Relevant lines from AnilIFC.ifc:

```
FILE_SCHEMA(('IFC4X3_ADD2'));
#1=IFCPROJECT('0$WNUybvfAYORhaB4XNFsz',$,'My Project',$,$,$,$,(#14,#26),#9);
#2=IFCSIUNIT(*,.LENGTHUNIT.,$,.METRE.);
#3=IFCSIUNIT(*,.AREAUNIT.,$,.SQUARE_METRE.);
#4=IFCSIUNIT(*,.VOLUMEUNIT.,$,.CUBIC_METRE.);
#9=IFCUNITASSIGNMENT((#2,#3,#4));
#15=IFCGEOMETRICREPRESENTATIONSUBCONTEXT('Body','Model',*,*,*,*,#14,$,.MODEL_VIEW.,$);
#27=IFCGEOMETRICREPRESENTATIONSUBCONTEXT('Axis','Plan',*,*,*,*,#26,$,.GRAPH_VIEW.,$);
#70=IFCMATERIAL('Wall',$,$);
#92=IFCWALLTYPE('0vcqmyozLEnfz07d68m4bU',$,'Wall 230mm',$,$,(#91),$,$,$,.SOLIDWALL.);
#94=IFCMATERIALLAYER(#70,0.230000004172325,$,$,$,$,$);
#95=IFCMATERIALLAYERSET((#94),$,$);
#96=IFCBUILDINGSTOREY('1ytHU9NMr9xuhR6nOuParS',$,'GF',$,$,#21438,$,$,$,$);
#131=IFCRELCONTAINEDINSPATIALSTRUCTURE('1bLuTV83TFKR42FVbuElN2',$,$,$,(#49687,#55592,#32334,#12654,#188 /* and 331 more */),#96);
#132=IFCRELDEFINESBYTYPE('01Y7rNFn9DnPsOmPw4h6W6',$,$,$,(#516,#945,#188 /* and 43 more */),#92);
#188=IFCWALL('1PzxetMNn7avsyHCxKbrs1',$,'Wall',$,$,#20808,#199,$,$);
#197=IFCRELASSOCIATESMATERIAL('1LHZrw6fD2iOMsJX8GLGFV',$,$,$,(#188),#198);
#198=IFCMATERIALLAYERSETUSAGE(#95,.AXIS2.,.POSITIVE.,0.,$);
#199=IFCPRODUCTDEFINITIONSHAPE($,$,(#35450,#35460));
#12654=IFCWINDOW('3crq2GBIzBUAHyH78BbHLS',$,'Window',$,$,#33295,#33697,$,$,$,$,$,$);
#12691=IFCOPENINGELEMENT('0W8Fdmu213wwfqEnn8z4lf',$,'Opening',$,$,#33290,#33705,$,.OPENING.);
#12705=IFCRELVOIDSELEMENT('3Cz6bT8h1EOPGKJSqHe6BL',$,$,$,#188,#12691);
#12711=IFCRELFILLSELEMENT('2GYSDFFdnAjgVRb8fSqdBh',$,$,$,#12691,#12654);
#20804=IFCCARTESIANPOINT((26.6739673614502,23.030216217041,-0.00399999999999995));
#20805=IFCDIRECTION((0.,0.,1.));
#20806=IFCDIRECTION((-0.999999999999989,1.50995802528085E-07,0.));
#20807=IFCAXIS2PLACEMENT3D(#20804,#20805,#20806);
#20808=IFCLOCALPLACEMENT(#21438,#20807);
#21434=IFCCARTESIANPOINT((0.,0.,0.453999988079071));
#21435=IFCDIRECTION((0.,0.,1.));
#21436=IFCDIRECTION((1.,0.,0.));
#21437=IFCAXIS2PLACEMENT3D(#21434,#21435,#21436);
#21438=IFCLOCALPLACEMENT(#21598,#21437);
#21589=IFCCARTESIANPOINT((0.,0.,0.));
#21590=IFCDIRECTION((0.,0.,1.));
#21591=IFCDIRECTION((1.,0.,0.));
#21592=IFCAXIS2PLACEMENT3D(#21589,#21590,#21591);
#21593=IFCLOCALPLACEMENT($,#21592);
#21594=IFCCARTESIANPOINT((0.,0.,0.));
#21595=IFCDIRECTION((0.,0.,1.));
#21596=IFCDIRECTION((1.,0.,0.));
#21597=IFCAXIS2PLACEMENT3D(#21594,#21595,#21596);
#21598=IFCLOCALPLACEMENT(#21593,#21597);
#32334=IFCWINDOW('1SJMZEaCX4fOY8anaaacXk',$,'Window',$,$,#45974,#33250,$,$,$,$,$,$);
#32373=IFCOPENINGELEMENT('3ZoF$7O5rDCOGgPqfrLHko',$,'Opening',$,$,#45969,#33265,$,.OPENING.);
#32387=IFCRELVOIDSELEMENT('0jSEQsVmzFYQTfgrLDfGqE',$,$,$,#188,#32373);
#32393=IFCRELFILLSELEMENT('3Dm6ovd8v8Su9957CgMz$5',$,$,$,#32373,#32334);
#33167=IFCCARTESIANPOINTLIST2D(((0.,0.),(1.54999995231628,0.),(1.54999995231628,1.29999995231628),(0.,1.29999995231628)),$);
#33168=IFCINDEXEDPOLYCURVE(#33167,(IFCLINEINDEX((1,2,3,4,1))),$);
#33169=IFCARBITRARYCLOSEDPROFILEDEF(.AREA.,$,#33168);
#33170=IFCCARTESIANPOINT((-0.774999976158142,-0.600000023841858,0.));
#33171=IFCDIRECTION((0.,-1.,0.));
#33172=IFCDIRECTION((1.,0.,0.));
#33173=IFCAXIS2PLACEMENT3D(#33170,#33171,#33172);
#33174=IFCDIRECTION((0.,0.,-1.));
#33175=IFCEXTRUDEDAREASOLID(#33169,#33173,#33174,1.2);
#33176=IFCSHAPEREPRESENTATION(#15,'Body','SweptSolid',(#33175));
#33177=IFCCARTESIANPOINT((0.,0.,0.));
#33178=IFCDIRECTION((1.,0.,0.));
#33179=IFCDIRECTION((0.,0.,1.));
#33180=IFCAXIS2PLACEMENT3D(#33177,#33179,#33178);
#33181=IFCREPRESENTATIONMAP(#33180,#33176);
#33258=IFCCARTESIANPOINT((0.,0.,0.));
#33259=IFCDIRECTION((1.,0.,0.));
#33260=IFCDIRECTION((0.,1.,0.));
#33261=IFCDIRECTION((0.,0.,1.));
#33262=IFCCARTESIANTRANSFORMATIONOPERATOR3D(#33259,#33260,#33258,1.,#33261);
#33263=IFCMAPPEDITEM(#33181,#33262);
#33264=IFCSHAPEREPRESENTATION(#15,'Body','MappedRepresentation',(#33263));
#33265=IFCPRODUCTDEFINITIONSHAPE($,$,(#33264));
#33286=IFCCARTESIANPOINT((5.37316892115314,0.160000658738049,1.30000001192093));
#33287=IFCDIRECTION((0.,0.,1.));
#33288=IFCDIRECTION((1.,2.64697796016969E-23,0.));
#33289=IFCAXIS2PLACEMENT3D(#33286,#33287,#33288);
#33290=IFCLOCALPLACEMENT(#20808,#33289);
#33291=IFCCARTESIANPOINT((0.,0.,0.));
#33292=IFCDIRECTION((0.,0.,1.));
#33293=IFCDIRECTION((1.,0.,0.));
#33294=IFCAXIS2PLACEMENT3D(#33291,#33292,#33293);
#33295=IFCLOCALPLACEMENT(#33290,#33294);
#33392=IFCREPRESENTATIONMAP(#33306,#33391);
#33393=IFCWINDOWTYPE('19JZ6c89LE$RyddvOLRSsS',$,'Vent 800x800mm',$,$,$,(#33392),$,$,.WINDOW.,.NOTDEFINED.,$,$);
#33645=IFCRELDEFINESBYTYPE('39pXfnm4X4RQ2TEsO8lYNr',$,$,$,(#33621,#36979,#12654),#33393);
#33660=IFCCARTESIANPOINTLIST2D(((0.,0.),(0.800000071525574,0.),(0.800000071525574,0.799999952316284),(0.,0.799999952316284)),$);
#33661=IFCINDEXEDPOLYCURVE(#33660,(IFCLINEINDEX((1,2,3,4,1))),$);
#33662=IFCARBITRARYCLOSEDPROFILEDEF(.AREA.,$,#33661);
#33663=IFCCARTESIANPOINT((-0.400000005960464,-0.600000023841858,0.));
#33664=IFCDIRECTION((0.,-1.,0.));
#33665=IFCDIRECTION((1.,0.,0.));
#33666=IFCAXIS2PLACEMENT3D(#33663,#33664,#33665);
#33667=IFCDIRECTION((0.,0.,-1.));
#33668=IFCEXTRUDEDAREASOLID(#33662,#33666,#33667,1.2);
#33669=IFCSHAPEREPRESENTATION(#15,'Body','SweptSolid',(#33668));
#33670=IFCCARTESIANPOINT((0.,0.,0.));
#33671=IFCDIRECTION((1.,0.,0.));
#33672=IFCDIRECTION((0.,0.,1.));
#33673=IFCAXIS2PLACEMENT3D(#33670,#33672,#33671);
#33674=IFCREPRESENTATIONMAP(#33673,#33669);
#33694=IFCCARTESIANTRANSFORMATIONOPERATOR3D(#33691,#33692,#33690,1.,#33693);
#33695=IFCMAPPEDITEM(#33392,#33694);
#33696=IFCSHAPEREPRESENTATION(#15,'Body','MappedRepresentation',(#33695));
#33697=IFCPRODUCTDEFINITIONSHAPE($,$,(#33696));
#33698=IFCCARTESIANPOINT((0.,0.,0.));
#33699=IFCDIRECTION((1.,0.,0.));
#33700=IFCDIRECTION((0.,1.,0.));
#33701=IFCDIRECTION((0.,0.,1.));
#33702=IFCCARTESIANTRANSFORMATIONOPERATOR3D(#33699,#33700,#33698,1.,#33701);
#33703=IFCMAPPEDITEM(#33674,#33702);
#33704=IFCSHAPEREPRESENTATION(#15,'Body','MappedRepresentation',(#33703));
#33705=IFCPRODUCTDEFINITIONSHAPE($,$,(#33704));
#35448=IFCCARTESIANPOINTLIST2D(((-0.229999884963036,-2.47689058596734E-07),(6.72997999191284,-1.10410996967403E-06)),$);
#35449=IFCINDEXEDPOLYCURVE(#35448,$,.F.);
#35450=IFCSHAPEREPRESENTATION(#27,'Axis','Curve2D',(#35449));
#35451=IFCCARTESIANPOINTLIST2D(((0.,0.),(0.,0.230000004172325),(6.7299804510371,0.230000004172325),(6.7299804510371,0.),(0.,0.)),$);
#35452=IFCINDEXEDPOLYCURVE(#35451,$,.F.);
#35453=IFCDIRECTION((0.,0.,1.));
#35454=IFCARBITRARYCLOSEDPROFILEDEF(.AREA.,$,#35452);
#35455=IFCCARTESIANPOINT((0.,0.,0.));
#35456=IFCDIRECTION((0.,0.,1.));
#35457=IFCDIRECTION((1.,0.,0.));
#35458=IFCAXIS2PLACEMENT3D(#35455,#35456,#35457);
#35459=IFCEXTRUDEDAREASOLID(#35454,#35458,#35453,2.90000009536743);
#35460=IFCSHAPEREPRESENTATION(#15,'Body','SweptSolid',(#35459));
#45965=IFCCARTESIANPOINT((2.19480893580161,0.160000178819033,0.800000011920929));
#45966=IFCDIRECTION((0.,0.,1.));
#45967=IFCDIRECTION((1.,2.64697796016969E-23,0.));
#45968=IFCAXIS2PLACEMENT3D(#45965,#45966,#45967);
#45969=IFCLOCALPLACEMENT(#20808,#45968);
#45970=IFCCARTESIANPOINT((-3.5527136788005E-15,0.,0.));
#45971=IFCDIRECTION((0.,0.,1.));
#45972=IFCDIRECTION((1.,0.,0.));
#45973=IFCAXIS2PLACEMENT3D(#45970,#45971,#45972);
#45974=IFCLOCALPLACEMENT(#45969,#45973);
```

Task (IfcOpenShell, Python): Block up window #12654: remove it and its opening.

```python
import ifcopenshell
import ifcopenshell.api.feature
import ifcopenshell.api.root
import ifcopenshell.geom
import ifcopenshell.util.shape

model = ifcopenshell.open("AnilIFC.ifc")
settings = ifcopenshell.geom.settings()


def volume(element):
    """Net volume in cubic metres, openings subtracted."""
    shape = ifcopenshell.geom.create_shape(settings, element)
    return ifcopenshell.util.shape.get_volume(shape.geometry)


window = model.by_id(12654)
opening = window.FillsVoids[0].RelatingOpeningElement
wall = opening.VoidsElements[0].RelatingBuildingElement
before = volume(wall)

ifcopenshell.api.root.remove_product(model, product=window)
ifcopenshell.api.feature.remove_feature(model, feature=opening)

after = volume(wall)

print(f"wall volume {before:.3f} -> {after:.3f} m3")

model.write("AnilIFC_rev.ifc")
```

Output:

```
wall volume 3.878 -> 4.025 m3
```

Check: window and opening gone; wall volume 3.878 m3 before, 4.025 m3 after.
